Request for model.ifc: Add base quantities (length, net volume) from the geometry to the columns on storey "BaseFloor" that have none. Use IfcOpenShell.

First a look at what the model holds.

```python
import ifcopenshell
import ifcopenshell.util.element
import ifcopenshell.util.unit

model = ifcopenshell.open("model.ifc")
print(model.schema)
for unit_type in ("LENGTHUNIT", "AREAUNIT", "VOLUMEUNIT"):
    print(unit_type, ifcopenshell.util.unit.calculate_unit_scale(model, unit_type))
storey = next(s for s in model.by_type("IfcBuildingStorey") if s.Name == "BaseFloor")
columns = [e for e in ifcopenshell.util.element.get_decomposition(storey) if e.is_a("IfcColumn")]
for e in sorted(columns, key=lambda e: e.id()):
    print(e.id(), e.is_a(), e.Name, list(ifcopenshell.util.element.get_psets(e, qtos_only=True)), sep=" | ")
```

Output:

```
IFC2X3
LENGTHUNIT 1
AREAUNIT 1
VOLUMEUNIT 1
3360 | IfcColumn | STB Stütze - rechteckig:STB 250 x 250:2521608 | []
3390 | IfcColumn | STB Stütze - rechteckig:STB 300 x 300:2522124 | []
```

```python
import ifcopenshell
import ifcopenshell.api.pset
import ifcopenshell.geom
import ifcopenshell.util.element
import ifcopenshell.util.shape
import ifcopenshell.util.unit

model = ifcopenshell.open("model.ifc")
unit_scale = ifcopenshell.util.unit.calculate_unit_scale(model)
volume_scale = ifcopenshell.util.unit.calculate_unit_scale(model, "VOLUMEUNIT")
settings = ifcopenshell.geom.settings()

storey = next(s for s in model.by_type("IfcBuildingStorey") if s.Name == "BaseFloor")
columns = [e for e in ifcopenshell.util.element.get_decomposition(storey) if e.is_a("IfcColumn")]

for e in sorted(columns, key=lambda e: e.id()):
    if ifcopenshell.util.element.get_psets(e, qtos_only=True, should_inherit=False):
        continue
    # Geometry comes back in metres, in the element's own axes.
    shape = ifcopenshell.geom.create_shape(settings, e)
    values = {
        "Length": ifcopenshell.util.shape.get_z(shape.geometry) / unit_scale,
        "NetVolume": ifcopenshell.util.shape.get_volume(shape.geometry) / volume_scale,
    }
    qto = ifcopenshell.api.pset.add_qto(model, product=e, name="BaseQuantities")
    ifcopenshell.api.pset.edit_qto(model, qto=qto, properties=values)
    print(e.id(), {k: round(v, 3) for k, v in values.items()})

model.write("model_rev.ifc")
```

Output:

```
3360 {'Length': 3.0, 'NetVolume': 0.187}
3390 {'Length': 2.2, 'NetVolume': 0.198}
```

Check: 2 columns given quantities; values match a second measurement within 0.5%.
